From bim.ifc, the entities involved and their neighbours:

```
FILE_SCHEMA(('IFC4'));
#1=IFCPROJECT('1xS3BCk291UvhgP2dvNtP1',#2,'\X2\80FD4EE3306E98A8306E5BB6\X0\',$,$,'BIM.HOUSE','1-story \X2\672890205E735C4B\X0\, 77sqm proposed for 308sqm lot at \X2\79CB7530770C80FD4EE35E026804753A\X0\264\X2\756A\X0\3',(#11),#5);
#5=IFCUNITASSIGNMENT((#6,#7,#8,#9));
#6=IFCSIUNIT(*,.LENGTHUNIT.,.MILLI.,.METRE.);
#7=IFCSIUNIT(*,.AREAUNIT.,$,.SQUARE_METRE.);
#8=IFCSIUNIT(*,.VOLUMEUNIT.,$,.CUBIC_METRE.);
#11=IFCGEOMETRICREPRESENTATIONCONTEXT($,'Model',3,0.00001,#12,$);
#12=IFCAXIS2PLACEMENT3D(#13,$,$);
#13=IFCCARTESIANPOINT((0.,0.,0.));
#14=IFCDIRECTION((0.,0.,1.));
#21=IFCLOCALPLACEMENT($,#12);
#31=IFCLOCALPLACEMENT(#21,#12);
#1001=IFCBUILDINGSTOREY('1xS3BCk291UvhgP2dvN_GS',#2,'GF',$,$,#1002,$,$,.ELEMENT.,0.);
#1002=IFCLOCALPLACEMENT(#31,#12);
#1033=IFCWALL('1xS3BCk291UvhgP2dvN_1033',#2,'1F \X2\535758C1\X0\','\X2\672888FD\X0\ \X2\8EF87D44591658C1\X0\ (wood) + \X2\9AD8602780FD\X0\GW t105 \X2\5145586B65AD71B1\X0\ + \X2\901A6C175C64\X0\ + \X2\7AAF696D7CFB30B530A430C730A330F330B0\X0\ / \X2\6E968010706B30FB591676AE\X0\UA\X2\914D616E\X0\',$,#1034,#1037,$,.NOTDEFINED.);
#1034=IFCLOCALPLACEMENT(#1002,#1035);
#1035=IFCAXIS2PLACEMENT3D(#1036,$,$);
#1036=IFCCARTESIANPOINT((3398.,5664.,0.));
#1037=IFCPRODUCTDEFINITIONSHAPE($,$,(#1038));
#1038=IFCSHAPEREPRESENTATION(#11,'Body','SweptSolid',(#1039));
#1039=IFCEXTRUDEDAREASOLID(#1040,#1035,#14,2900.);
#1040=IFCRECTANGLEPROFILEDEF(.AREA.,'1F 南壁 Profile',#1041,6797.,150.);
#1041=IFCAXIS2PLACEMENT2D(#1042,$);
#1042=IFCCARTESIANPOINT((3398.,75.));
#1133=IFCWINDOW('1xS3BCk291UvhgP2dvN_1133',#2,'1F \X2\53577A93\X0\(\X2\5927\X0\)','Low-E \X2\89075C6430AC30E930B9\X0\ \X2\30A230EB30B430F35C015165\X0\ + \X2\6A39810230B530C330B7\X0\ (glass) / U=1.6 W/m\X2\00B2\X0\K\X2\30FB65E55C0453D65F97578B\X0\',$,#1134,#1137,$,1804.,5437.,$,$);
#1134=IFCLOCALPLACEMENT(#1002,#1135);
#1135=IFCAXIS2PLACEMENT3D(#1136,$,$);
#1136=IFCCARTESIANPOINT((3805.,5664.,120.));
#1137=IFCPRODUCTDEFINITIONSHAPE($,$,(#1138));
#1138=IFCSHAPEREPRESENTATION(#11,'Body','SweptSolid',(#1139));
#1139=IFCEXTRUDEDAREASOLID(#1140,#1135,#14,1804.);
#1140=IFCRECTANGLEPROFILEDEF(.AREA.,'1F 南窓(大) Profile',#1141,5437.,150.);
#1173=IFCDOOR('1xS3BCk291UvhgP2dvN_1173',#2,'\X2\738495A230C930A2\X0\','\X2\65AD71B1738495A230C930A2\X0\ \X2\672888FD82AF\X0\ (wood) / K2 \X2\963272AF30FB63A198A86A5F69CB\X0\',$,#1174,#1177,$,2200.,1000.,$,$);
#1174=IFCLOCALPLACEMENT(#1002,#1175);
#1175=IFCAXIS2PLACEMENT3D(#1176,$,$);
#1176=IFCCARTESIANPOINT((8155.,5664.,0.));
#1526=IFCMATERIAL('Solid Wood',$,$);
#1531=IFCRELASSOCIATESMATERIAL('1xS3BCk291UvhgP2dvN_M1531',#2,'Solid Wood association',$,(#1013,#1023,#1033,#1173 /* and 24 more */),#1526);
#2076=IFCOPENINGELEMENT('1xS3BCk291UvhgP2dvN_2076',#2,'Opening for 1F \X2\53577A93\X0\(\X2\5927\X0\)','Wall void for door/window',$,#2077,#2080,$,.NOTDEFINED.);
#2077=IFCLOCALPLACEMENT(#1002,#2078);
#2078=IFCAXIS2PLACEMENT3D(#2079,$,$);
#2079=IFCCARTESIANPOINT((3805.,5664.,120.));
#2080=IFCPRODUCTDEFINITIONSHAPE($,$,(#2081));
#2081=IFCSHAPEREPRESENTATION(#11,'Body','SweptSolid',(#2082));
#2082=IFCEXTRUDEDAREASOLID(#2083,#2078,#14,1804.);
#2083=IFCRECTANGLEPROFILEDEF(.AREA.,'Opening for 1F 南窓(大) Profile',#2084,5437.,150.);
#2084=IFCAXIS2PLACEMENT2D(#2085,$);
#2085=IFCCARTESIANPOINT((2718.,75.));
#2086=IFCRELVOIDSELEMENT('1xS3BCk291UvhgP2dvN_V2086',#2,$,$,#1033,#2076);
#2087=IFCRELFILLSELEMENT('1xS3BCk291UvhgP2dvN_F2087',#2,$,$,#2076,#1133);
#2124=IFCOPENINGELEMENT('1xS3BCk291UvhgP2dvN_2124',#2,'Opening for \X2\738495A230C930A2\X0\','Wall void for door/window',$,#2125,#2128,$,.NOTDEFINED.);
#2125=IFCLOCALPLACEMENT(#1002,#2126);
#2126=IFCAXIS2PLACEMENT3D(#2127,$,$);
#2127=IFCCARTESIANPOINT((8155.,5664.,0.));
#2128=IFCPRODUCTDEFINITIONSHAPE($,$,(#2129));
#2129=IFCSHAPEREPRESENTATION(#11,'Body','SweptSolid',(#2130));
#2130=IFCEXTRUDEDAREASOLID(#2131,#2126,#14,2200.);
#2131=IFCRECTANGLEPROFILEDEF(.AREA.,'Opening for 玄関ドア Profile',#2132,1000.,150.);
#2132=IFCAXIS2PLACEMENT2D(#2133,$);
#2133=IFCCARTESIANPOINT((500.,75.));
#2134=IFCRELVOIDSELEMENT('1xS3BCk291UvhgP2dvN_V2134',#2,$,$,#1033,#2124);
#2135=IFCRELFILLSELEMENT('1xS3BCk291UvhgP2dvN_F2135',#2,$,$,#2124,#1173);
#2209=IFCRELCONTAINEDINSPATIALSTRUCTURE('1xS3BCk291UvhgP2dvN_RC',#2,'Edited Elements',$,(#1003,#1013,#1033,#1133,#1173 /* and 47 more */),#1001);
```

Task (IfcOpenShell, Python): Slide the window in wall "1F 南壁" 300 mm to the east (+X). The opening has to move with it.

```python
import ifcopenshell
import ifcopenshell.api.geometry
import ifcopenshell.util.placement
import ifcopenshell.util.unit

model = ifcopenshell.open("bim.ifc")
unit_scale = ifcopenshell.util.unit.calculate_unit_scale(model)

window = model.by_guid("1xS3BCk291UvhgP2dvN_1133")
opening = window.FillsVoids[0].RelatingOpeningElement
wall = opening.VoidsElements[0].RelatingBuildingElement

wall_matrix = ifcopenshell.util.placement.get_local_placement(wall.ObjectPlacement)
shift = wall_matrix[:3, 0] * 0.3 / unit_scale
before = ifcopenshell.util.placement.get_local_placement(window.ObjectPlacement)[:3, 3].copy()

# The window is not placed relative to its opening, so move both.
for product in (opening, window):
    matrix = ifcopenshell.util.placement.get_local_placement(product.ObjectPlacement)
    matrix[:3, 3] += shift
    ifcopenshell.api.geometry.edit_object_placement(model, product=product, matrix=matrix, is_si=False)

after = ifcopenshell.util.placement.get_local_placement(window.ObjectPlacement)[:3, 3]
print("window moved by", (after - before).round(3) + 0.0)

model.write("bim-out.ifc")
```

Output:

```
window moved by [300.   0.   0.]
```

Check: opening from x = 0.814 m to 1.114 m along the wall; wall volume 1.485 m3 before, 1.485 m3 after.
